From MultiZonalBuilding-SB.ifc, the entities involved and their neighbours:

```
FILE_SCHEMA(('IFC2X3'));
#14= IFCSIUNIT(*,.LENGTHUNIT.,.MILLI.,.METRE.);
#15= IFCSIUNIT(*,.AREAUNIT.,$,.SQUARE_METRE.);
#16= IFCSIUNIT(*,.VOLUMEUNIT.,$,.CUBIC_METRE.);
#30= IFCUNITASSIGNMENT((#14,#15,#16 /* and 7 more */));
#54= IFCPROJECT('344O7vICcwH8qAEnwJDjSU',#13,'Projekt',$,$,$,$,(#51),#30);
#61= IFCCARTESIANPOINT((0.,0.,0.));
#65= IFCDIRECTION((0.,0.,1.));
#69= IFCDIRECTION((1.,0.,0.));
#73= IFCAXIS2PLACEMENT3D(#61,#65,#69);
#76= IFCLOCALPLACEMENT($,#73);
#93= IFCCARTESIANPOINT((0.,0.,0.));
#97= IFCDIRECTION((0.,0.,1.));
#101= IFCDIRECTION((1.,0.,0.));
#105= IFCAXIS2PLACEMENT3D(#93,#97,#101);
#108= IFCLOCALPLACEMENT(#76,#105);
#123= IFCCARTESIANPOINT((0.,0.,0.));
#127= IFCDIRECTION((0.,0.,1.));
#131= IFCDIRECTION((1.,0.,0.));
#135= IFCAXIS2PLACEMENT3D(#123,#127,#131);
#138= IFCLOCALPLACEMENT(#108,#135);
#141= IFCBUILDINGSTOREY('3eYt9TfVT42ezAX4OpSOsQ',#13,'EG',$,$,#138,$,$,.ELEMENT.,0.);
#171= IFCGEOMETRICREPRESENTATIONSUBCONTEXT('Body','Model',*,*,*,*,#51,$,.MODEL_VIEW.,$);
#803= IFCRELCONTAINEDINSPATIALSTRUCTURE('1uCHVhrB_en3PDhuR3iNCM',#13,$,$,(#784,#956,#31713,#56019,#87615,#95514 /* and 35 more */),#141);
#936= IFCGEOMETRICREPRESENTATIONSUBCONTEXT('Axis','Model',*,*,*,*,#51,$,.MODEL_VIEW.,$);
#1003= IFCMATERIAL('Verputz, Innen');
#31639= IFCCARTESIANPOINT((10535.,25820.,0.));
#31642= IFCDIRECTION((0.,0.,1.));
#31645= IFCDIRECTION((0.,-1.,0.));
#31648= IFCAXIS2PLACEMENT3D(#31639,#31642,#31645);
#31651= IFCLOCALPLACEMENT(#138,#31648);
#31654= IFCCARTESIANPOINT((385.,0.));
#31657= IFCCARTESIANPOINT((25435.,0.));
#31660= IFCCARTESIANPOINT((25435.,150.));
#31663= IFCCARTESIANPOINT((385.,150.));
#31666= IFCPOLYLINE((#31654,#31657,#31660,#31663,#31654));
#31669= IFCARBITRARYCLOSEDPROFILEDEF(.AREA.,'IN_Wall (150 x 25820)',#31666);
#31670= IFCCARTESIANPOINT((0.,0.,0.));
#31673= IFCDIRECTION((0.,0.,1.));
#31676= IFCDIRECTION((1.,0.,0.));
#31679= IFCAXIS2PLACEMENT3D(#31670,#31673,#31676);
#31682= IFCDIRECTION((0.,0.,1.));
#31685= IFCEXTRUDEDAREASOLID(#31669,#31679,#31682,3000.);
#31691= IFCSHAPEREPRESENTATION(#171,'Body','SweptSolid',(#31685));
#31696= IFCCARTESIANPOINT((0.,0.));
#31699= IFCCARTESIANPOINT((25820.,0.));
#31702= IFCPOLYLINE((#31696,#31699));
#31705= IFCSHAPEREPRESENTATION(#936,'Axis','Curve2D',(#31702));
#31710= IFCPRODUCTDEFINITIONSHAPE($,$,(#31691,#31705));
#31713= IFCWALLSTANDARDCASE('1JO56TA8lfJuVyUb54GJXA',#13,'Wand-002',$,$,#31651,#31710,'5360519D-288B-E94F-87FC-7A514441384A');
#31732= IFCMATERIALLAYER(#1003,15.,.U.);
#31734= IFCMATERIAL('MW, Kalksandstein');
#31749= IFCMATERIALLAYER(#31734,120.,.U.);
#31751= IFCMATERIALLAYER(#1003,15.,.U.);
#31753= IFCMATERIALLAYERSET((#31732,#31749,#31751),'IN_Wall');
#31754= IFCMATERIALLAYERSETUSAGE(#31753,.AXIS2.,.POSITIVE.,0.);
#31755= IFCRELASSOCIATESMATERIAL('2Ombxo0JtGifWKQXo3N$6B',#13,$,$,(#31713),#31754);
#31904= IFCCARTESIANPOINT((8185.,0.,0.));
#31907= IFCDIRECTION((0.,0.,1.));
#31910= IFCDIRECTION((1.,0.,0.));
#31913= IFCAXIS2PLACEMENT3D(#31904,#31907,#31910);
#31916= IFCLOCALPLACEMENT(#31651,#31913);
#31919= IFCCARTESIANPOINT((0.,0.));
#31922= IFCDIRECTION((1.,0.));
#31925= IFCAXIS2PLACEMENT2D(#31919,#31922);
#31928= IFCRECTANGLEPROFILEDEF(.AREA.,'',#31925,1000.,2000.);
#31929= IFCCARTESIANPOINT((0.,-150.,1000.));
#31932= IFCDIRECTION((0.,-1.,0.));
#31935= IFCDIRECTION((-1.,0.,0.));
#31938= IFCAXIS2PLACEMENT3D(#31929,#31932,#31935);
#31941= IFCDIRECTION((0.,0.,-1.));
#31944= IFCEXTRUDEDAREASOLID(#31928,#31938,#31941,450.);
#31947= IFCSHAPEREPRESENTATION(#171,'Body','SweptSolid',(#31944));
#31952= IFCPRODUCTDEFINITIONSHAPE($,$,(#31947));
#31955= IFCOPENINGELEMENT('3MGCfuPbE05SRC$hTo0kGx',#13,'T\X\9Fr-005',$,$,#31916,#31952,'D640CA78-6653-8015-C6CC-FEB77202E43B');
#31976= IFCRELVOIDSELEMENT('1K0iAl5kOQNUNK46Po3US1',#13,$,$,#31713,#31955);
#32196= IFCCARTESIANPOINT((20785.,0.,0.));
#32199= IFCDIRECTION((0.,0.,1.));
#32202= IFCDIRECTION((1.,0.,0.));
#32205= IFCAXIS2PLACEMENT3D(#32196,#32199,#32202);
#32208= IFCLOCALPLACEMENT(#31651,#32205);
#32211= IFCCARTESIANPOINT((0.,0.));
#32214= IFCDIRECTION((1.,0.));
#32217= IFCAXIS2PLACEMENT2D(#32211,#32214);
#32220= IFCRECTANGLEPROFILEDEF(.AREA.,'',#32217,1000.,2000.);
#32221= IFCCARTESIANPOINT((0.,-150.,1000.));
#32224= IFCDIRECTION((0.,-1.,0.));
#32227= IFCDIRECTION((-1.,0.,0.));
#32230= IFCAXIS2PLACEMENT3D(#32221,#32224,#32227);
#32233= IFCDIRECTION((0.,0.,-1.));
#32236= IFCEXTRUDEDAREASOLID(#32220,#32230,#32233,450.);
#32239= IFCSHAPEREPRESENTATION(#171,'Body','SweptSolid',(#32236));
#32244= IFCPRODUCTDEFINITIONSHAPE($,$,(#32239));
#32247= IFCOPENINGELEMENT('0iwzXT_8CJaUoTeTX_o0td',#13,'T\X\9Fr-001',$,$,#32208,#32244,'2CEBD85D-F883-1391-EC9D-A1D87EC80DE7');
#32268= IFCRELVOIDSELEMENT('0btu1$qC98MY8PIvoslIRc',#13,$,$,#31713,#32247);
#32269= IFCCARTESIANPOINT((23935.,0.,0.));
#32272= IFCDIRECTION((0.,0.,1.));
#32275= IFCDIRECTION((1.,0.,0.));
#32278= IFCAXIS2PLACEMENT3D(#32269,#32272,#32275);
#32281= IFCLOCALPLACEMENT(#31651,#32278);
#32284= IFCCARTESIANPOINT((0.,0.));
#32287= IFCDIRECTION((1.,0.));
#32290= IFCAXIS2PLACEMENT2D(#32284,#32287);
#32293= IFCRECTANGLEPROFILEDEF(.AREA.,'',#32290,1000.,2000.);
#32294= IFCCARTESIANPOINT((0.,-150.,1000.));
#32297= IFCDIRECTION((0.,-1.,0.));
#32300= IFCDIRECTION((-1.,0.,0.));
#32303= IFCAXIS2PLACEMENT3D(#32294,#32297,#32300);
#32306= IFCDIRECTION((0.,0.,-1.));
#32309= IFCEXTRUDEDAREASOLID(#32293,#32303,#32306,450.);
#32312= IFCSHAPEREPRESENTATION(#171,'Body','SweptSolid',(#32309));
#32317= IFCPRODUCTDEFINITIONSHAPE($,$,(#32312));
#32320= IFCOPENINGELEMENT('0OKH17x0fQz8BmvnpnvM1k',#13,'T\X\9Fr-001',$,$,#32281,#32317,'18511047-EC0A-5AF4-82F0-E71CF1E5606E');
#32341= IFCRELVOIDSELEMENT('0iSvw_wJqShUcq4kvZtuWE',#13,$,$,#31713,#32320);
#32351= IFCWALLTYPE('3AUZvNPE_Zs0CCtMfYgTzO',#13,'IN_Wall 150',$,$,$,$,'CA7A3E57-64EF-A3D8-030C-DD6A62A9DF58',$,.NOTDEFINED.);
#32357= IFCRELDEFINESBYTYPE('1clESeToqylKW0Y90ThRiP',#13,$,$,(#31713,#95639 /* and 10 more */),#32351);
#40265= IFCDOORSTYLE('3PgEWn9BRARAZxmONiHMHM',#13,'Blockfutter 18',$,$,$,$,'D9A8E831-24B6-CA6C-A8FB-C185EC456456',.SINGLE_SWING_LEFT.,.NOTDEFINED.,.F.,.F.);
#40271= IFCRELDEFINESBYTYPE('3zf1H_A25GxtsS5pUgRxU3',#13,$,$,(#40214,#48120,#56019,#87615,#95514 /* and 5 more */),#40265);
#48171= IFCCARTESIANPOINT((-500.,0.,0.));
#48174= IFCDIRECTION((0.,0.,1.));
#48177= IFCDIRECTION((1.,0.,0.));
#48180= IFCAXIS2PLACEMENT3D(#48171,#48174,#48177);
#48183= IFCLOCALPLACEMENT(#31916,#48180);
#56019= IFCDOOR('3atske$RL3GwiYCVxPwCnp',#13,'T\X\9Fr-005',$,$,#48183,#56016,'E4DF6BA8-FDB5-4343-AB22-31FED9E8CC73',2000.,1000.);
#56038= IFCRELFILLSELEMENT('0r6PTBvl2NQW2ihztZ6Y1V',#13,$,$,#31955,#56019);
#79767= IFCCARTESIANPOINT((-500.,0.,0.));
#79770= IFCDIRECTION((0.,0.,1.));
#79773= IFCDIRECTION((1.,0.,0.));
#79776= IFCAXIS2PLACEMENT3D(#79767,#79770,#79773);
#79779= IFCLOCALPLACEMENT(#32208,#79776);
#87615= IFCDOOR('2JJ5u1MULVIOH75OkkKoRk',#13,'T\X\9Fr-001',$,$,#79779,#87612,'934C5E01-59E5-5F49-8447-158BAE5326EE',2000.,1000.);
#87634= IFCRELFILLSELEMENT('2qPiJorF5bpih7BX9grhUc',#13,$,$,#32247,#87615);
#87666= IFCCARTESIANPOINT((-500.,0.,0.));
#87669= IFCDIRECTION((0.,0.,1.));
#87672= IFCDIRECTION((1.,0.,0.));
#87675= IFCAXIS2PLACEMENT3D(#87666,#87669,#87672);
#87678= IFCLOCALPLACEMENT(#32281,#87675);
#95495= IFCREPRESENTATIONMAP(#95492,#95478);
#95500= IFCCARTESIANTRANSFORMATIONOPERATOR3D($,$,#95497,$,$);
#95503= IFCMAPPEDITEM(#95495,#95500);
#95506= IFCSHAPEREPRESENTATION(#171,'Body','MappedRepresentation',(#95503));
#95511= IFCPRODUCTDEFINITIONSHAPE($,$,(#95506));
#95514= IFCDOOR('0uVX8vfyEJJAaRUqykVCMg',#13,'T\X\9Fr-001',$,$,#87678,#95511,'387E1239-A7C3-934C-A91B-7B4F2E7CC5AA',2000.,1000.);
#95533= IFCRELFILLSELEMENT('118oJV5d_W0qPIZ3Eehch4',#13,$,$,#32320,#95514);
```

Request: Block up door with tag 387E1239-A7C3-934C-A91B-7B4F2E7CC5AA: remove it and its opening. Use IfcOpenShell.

```python
import ifcopenshell
import ifcopenshell.api.feature
import ifcopenshell.api.root
import ifcopenshell.geom
import ifcopenshell.util.shape

model = ifcopenshell.open("MultiZonalBuilding-SB.ifc")
settings = ifcopenshell.geom.settings()


def volume(element):
    """Net volume in cubic metres, openings subtracted."""
    shape = ifcopenshell.geom.create_shape(settings, element)
    return ifcopenshell.util.shape.get_volume(shape.geometry)


door = model.by_id(95514)
opening = door.FillsVoids[0].RelatingOpeningElement
wall = opening.VoidsElements[0].RelatingBuildingElement
before = volume(wall)

ifcopenshell.api.root.remove_product(model, product=door)
ifcopenshell.api.feature.remove_feature(model, feature=opening)

after = volume(wall)

print(f"wall volume {before:.3f} -> {after:.3f} m3")

model.write("MultiZonalBuilding-SB_rev.ifc")
```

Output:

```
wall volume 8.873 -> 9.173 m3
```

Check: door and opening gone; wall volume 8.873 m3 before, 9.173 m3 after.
